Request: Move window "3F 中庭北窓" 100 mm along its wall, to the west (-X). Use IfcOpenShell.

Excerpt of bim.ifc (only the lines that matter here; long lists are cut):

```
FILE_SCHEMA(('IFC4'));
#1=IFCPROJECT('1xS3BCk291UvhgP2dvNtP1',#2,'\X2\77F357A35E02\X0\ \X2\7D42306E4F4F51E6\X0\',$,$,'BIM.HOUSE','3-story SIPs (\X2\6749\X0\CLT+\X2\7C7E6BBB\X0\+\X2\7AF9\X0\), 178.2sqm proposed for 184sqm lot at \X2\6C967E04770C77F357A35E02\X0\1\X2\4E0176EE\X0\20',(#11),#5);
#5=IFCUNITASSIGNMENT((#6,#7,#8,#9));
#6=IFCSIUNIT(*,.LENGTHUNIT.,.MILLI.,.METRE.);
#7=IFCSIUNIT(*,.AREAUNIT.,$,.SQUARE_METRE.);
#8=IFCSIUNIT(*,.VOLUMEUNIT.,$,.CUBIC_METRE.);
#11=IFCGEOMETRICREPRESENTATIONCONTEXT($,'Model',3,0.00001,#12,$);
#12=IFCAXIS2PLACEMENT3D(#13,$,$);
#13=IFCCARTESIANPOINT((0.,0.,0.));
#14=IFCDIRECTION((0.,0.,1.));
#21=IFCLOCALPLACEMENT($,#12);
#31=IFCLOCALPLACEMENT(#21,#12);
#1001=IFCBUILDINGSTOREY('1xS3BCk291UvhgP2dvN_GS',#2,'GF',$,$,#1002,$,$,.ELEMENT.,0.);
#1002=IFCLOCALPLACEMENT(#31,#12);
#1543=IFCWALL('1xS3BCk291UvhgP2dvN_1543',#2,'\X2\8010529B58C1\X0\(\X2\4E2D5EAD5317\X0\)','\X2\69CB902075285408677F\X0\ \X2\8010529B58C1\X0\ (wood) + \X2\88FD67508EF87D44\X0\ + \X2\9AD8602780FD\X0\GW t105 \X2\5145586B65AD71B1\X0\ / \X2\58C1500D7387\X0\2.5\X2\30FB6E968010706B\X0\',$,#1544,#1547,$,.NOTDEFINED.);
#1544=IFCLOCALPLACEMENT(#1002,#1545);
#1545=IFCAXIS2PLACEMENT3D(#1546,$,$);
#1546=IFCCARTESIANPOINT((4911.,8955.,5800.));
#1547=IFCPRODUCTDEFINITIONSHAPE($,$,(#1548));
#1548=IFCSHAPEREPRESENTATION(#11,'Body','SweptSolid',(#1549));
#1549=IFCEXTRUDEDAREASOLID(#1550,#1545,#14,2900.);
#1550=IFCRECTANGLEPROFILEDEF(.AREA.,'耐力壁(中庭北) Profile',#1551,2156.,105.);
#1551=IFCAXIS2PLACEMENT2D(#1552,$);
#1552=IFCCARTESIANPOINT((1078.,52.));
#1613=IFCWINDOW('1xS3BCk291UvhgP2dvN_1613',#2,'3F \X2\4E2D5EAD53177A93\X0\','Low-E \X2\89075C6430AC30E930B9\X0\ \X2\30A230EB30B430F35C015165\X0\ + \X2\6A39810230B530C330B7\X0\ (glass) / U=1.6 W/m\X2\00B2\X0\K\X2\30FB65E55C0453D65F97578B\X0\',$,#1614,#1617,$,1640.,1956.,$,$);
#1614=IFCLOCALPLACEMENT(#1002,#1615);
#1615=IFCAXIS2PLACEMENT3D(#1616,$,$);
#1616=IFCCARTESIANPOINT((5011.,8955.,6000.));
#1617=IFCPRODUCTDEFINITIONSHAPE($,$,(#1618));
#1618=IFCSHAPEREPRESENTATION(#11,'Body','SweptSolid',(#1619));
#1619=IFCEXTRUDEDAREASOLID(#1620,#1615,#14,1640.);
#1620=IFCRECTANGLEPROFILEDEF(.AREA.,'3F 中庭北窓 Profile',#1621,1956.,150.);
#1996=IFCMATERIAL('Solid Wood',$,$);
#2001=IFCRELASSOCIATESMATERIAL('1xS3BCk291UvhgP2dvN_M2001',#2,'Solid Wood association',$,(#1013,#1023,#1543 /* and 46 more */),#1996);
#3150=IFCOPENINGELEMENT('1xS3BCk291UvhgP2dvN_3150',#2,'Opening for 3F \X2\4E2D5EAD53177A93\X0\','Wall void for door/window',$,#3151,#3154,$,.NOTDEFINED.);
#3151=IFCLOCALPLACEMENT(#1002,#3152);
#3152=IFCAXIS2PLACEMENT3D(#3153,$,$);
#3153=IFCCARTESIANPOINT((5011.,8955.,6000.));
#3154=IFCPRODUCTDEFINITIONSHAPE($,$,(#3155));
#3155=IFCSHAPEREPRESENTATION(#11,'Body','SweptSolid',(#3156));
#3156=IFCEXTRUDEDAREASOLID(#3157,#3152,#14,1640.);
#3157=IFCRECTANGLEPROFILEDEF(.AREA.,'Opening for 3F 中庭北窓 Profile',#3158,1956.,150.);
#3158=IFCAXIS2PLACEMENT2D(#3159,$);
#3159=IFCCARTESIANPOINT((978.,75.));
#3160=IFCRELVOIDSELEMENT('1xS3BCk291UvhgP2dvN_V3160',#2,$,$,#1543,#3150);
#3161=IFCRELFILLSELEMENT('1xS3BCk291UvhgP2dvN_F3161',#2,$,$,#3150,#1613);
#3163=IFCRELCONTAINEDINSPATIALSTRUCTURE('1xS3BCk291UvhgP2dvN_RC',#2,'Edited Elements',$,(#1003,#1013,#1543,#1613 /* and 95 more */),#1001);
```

```python
import ifcopenshell
import ifcopenshell.api.geometry
import ifcopenshell.util.placement
import ifcopenshell.util.unit

model = ifcopenshell.open("bim.ifc")
unit_scale = ifcopenshell.util.unit.calculate_unit_scale(model)

window = model.by_id(1613)
opening = window.FillsVoids[0].RelatingOpeningElement
wall = opening.VoidsElements[0].RelatingBuildingElement

wall_matrix = ifcopenshell.util.placement.get_local_placement(wall.ObjectPlacement)
shift = wall_matrix[:3, 0] * -0.1 / unit_scale
before = ifcopenshell.util.placement.get_local_placement(window.ObjectPlacement)[:3, 3].copy()

# The window is not placed relative to its opening, so move both.
for product in (opening, window):
    matrix = ifcopenshell.util.placement.get_local_placement(product.ObjectPlacement)
    matrix[:3, 3] += shift
    ifcopenshell.api.geometry.edit_object_placement(model, product=product, matrix=matrix, is_si=False)

after = ifcopenshell.util.placement.get_local_placement(window.ObjectPlacement)[:3, 3]
print("window moved by", (after - before).round(3) + 0.0)

model.write("bim_edited.ifc")
```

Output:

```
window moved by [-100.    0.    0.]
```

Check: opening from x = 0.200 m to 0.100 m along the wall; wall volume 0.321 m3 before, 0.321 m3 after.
